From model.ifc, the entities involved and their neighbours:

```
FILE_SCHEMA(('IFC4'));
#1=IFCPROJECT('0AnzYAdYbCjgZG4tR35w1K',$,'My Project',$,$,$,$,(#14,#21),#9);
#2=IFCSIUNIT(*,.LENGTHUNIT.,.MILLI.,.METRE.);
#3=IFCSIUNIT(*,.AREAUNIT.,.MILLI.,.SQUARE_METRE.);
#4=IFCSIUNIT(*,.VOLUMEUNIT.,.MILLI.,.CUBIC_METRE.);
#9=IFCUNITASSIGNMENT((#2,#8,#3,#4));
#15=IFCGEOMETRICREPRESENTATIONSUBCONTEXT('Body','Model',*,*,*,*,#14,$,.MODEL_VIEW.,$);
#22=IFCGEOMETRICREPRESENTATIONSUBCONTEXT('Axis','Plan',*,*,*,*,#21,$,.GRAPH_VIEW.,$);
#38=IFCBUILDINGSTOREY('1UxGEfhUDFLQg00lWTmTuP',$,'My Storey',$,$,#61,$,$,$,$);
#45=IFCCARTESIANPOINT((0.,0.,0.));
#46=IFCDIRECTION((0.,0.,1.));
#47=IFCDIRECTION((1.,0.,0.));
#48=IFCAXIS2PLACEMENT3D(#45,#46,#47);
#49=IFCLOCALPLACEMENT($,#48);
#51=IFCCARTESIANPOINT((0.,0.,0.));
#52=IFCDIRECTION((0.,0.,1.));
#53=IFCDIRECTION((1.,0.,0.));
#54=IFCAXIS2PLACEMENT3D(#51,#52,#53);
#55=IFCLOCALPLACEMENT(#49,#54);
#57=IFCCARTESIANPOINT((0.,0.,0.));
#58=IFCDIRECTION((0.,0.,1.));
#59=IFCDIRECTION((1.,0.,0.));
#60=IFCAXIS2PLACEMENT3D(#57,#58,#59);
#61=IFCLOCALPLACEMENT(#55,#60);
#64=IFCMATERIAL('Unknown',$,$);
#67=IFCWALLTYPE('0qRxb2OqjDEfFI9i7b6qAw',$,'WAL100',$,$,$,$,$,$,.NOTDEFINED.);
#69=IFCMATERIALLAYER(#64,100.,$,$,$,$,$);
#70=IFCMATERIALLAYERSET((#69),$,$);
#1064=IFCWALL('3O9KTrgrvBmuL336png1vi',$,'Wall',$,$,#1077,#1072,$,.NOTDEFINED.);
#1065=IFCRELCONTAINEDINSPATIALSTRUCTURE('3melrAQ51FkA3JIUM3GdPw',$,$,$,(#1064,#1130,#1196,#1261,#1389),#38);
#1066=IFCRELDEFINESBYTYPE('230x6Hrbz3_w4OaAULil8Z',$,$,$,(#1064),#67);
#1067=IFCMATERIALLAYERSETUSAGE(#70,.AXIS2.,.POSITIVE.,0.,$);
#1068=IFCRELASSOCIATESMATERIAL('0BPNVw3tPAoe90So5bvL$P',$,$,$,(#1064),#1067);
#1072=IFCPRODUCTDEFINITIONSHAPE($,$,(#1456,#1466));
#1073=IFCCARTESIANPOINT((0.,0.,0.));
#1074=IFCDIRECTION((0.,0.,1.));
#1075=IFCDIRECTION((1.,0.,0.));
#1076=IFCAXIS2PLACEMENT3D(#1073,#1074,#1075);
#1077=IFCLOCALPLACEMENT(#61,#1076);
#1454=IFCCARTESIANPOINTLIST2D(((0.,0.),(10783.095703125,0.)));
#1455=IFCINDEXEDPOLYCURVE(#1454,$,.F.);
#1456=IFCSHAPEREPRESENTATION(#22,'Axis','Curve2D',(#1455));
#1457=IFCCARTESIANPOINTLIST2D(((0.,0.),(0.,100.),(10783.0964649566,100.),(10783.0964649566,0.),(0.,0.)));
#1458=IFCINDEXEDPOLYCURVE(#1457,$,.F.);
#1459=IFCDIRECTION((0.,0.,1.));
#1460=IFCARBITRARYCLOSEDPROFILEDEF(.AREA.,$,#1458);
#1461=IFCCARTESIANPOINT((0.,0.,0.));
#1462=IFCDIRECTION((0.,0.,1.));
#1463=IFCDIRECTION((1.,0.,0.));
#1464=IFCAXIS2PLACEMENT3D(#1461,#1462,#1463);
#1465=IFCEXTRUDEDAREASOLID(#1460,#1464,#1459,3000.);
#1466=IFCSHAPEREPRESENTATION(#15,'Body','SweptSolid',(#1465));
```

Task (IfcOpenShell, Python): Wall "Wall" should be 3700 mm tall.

```python
import ifcopenshell
import ifcopenshell.geom
import ifcopenshell.util.representation
import ifcopenshell.util.shape

model = ifcopenshell.open("model.ifc")
settings = ifcopenshell.geom.settings()


def volume(element):
    """Net volume in cubic metres, openings subtracted."""
    shape = ifcopenshell.geom.create_shape(settings, element)
    return ifcopenshell.util.shape.get_volume(shape.geometry)


wall = model.by_guid("3O9KTrgrvBmuL336png1vi")
before = volume(wall)

body = ifcopenshell.util.representation.get_representation(wall, "Model", "Body")
solid = body.Items[0]
old_height = solid.Depth
solid.Depth = 3700.0
after = volume(wall)

print(f"height {old_height:g} -> {solid.Depth:g}, volume {before:.3f} -> {after:.3f} m3")

model.write("model_updated.ifc")
```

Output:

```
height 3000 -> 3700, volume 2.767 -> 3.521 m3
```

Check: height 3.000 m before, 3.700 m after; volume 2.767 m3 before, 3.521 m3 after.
